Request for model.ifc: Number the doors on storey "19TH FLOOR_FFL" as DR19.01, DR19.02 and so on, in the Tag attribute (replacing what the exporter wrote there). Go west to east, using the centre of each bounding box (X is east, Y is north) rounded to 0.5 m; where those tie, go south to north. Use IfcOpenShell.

First a look at what the model holds.

```python
import ifcopenshell
import ifcopenshell.util.element
import ifcopenshell.util.placement

model = ifcopenshell.open("model.ifc")
print(model.schema)
storey = next(s for s in model.by_type("IfcBuildingStorey") if s.Name == "19TH FLOOR_FFL")
doors = [e for e in ifcopenshell.util.element.get_decomposition(storey) if e.is_a("IfcDoor")]
for e in sorted(doors, key=lambda e: e.id()):
    origin = ifcopenshell.util.placement.get_local_placement(e.ObjectPlacement)[:3, 3]
    print(e.id(), e.Tag, e.Name, origin.round(2) + 0.0, sep=" | ")
```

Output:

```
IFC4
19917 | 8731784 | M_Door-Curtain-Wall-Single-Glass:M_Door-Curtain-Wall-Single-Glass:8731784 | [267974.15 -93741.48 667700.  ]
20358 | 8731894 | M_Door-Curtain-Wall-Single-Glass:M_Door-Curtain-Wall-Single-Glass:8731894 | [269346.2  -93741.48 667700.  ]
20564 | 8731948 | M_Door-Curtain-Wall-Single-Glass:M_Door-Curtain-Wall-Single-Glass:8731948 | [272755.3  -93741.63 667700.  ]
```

```python
import ifcopenshell
import ifcopenshell.geom
import ifcopenshell.util.element
import ifcopenshell.util.shape

model = ifcopenshell.open("model.ifc")
settings = ifcopenshell.geom.settings()
settings.set("use-world-coords", True)


def centre(element):
    shape = ifcopenshell.geom.create_shape(settings, element)
    return ifcopenshell.util.shape.get_bbox_centroid(shape.geometry)


storey = next(s for s in model.by_type("IfcBuildingStorey") if s.Name == "19TH FLOOR_FFL")
doors = [e for e in ifcopenshell.util.element.get_decomposition(storey) if e.is_a("IfcDoor")]

# Insertion points can sit at a corner or the storey origin, so sort by the geometry (in metres).
centres = {e: centre(e) for e in doors}
doors.sort(key=lambda e: (round(centres[e][0] / 0.5), centres[e][1]))

for i, e in enumerate(doors, start=1):
    number = f"DR19.{i:02d}"
    e.Tag = number
    print(e.id(), number)

model.write("model-out.ifc")
```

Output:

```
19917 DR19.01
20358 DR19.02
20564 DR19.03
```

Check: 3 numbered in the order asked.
